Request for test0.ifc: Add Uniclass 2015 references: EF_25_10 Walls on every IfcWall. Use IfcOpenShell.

First a look at what the model holds.

```python
import ifcopenshell

model = ifcopenshell.open("test0.ifc")
print(model.schema)
print("classifications:", [c.Name for c in model.by_type("IfcClassification")])
for ifc_class in ("IfcDoor", "IfcRoof", "IfcStair", "IfcWall", "IfcWindow"):
    print(ifc_class, len(model.by_type(ifc_class)))
```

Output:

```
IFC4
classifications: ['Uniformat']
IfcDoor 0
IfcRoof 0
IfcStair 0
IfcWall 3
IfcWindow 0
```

```python
import ifcopenshell
import ifcopenshell.api.classification

model = ifcopenshell.open("test0.ifc")

system = ifcopenshell.api.classification.add_classification(model, classification="Uniclass 2015")

codes = {
    "IfcWall": ("EF_25_10", "Walls"),
}
for ifc_class, (code, name) in codes.items():
    products = model.by_type(ifc_class)
    ifcopenshell.api.classification.add_reference(
        model, products=products, classification=system, identification=code, name=name
    )
    print(code, len(products))

model.write("test0_edited.ifc")
```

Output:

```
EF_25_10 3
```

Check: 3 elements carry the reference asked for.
